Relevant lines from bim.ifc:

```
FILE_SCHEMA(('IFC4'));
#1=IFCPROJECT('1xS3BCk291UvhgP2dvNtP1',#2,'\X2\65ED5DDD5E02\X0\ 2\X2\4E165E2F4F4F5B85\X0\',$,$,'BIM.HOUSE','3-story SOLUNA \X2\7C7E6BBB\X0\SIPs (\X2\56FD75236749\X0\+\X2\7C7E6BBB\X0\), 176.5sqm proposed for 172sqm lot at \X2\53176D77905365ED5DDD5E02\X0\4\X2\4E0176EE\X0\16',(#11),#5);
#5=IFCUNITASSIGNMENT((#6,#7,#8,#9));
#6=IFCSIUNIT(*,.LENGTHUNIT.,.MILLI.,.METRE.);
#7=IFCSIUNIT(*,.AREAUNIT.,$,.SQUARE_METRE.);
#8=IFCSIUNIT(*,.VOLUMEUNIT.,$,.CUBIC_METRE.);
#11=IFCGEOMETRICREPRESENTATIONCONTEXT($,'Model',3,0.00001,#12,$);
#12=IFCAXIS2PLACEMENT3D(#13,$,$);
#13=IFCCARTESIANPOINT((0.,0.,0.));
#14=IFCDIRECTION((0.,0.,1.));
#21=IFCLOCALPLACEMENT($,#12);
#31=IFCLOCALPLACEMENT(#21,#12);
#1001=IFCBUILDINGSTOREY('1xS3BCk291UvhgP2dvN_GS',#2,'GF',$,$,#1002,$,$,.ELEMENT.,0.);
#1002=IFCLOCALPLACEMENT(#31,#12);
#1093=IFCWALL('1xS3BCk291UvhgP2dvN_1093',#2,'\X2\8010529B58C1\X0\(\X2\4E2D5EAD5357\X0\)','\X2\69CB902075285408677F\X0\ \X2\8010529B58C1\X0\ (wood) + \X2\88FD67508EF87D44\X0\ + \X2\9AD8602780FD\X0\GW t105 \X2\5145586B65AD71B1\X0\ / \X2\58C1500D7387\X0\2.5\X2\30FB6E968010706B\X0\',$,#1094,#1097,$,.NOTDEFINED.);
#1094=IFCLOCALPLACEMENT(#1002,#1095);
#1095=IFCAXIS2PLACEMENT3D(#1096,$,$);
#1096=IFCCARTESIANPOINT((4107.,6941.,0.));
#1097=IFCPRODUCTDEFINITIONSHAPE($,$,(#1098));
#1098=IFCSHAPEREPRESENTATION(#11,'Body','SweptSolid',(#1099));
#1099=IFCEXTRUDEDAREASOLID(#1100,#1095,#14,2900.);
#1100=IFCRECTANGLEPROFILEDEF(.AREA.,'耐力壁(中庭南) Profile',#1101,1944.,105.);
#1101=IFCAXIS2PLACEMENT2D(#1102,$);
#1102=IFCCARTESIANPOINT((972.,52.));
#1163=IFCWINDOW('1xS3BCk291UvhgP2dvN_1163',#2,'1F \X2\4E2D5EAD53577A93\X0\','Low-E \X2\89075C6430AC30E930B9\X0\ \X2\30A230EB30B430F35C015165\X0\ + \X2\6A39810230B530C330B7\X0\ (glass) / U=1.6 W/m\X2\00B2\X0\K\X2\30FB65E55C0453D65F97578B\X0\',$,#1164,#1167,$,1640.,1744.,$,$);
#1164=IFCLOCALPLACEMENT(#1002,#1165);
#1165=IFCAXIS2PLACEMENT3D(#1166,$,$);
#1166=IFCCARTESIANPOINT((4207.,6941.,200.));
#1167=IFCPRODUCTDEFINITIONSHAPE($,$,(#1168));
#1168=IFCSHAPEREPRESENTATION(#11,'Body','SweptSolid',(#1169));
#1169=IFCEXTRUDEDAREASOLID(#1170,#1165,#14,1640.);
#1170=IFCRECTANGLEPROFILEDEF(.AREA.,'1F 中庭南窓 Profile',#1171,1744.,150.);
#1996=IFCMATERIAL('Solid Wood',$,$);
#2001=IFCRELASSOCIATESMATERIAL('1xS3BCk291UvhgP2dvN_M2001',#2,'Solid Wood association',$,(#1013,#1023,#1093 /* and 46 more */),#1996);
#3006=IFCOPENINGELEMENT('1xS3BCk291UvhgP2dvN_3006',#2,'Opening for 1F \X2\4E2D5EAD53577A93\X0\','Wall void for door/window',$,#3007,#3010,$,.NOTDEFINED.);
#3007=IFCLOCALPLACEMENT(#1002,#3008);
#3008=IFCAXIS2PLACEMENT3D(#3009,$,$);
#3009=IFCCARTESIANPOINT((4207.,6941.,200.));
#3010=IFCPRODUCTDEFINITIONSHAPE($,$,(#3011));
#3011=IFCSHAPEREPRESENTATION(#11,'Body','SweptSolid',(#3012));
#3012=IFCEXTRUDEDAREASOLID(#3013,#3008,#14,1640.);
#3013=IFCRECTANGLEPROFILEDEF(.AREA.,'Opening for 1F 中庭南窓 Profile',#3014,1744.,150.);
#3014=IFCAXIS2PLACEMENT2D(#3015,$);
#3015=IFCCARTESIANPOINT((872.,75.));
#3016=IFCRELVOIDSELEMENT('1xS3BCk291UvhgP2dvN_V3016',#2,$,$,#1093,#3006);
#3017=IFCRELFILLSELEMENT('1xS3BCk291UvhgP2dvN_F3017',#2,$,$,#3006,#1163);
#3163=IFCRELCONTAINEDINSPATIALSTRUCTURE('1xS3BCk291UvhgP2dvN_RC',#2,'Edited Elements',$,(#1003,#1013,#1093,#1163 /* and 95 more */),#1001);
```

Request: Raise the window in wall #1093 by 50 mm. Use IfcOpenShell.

```python
import numpy as np
import ifcopenshell
import ifcopenshell.api.geometry
import ifcopenshell.util.placement
import ifcopenshell.util.unit

model = ifcopenshell.open("bim.ifc")
unit_scale = ifcopenshell.util.unit.calculate_unit_scale(model)

window = model.by_guid("1xS3BCk291UvhgP2dvN_1163")
opening = window.FillsVoids[0].RelatingOpeningElement
dz = 0.05 / unit_scale

shift = np.array([0.0, 0.0, dz])
# The window is not placed relative to its opening, so move both.
for product in (opening, window):
    matrix = ifcopenshell.util.placement.get_local_placement(product.ObjectPlacement)
    matrix[:3, 3] += shift
    ifcopenshell.api.geometry.edit_object_placement(model, product=product, matrix=matrix, is_si=False)

print(f"moved by {dz * unit_scale:+.3f} m")

model.write("bim_v2.ifc")
```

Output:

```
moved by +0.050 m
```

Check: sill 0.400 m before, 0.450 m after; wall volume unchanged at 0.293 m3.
